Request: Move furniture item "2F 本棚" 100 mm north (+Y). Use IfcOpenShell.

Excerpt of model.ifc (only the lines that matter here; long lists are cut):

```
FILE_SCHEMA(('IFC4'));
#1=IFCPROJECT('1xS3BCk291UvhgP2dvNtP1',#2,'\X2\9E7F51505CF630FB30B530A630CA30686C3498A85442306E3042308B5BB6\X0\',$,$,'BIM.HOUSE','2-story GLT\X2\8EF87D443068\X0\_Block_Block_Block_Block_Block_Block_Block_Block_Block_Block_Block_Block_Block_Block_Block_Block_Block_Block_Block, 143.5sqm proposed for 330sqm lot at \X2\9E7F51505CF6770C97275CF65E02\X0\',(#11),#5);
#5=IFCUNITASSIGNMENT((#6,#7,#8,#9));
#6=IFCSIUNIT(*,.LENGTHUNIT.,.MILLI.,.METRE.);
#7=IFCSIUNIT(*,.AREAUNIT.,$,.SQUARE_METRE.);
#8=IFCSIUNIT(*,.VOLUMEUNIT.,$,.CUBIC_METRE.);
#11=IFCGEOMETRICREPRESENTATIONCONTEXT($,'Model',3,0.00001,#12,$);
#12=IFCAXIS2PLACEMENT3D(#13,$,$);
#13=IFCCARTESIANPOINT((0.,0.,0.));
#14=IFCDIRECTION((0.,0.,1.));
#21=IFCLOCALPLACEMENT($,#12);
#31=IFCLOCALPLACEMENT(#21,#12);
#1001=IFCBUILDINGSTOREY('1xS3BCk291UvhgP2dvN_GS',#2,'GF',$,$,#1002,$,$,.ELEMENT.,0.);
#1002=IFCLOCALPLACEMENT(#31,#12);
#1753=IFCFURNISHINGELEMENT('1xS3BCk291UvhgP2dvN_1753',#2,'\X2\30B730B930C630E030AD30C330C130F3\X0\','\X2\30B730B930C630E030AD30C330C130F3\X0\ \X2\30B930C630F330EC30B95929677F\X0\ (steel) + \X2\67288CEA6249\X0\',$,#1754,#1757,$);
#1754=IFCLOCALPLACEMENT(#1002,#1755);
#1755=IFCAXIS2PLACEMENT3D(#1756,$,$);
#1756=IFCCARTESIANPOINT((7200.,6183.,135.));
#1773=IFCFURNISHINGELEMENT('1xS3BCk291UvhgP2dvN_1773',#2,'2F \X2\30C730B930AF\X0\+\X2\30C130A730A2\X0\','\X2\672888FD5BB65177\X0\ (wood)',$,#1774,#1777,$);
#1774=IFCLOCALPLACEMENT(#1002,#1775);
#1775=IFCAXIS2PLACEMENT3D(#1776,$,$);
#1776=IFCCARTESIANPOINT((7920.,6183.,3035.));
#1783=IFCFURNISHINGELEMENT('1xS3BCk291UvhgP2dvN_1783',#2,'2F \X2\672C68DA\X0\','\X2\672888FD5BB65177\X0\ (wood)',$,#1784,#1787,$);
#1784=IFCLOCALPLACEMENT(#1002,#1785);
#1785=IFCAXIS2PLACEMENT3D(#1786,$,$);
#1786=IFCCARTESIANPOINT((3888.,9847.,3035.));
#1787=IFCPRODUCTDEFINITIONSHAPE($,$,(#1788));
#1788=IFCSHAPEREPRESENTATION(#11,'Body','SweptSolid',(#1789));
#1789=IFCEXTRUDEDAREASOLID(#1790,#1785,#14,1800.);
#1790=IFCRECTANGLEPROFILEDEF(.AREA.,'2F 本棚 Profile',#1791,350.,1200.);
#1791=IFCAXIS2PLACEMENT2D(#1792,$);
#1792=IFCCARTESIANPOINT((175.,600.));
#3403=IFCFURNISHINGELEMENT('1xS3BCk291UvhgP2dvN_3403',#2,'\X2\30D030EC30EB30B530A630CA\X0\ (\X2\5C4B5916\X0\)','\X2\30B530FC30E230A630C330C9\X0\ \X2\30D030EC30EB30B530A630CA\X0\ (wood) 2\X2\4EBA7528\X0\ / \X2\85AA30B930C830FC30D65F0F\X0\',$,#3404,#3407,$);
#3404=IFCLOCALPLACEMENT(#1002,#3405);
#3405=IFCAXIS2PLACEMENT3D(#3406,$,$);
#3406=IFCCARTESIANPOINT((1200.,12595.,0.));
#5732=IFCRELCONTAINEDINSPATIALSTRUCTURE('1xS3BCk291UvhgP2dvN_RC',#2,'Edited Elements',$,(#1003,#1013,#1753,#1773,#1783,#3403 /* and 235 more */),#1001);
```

```python
import ifcopenshell
import ifcopenshell.api.geometry
import ifcopenshell.util.placement

model = ifcopenshell.open("model.ifc")

item = model.by_guid("1xS3BCk291UvhgP2dvN_1783")
matrix = ifcopenshell.util.placement.get_local_placement(item.ObjectPlacement)
matrix[1, 3] += 100.0
ifcopenshell.api.geometry.edit_object_placement(model, product=item, matrix=matrix, is_si=False)

print(ifcopenshell.util.placement.get_local_placement(item.ObjectPlacement).round(3) + 0.0)

model.write("model_v2.ifc")
```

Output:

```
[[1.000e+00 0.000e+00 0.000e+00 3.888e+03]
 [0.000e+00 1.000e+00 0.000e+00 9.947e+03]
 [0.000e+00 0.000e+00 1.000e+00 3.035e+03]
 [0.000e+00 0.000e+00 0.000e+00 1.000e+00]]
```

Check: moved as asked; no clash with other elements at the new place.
